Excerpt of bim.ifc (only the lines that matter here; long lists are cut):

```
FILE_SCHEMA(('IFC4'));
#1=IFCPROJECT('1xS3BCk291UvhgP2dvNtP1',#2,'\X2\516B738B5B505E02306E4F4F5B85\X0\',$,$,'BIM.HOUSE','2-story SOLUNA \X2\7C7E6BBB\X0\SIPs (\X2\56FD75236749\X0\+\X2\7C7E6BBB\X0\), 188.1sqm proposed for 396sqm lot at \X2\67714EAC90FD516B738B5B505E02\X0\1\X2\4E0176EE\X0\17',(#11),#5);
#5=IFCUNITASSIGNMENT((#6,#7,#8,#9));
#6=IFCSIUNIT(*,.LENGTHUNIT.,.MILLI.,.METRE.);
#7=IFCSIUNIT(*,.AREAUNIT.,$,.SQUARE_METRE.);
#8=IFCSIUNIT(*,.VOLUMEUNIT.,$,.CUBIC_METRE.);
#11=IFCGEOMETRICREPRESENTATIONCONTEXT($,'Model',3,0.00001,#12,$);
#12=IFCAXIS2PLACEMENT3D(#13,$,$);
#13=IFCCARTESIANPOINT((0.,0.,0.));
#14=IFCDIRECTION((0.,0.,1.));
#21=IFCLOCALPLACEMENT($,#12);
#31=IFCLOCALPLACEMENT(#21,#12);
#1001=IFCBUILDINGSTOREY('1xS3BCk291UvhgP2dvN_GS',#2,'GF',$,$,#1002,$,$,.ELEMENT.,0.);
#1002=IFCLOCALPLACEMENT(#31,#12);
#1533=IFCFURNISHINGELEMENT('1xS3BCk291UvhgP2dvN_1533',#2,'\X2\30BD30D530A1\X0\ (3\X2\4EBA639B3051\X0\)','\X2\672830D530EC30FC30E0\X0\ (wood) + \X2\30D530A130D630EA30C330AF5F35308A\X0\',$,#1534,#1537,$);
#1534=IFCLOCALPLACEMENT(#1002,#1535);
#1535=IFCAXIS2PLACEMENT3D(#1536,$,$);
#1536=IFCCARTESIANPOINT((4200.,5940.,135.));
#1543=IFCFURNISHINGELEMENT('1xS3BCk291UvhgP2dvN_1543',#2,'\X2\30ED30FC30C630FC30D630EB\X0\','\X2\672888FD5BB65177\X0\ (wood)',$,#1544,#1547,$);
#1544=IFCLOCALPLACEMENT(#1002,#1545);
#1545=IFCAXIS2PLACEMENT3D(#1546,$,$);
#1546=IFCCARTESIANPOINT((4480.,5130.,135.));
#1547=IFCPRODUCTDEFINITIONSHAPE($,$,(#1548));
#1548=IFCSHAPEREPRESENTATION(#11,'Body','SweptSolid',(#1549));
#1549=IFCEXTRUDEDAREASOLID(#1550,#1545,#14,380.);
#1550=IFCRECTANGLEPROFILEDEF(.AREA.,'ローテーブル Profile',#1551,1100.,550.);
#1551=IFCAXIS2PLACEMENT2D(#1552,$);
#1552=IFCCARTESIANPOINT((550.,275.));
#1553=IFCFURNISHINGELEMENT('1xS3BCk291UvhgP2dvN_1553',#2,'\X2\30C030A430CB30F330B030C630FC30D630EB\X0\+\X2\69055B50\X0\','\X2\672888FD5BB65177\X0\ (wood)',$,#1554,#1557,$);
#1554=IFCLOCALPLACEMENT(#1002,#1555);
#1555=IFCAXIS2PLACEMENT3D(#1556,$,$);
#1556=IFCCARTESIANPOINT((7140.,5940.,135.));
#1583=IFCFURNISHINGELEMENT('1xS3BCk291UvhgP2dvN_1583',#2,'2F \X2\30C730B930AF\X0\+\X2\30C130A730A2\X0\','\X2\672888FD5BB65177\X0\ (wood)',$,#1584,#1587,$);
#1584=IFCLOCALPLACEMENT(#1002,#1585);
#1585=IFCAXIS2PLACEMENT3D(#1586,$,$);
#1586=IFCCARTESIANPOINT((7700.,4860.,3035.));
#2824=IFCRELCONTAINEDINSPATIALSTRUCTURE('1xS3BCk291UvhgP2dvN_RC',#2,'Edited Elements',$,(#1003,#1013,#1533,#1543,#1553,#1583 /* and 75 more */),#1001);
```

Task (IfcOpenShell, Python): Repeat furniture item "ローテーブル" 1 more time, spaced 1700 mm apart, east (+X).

```python
import numpy as np
import ifcopenshell
import ifcopenshell.api.geometry
import ifcopenshell.api.root
import ifcopenshell.util.element
import ifcopenshell.util.placement
import ifcopenshell.util.unit

model = ifcopenshell.open("bim.ifc")
unit_scale = ifcopenshell.util.unit.calculate_unit_scale(model)


def reuse_history(source, copy):
    """copy_class also copies each property set's owner history, people and application; keep the originals."""
    for rel in copy.IsDefinedBy:
        if rel.is_a("IfcRelDefinesByProperties") and (history := rel.RelatingPropertyDefinition.OwnerHistory):
            rel.RelatingPropertyDefinition.OwnerHistory = source.OwnerHistory
            ifcopenshell.util.element.remove_deep2(model, history)


source = model.by_id(1543)
base = ifcopenshell.util.placement.get_local_placement(source.ObjectPlacement)
step = np.array([1.0, 0.0, 0.0]) * 1.7 / unit_scale

for i in range(1, 2):
    copy = ifcopenshell.api.root.copy_class(model, product=source)
    copy.Representation = ifcopenshell.util.element.copy_deep(
        model, source.Representation, exclude=["IfcGeometricRepresentationContext", "IfcRepresentationMap"]
    )
    reuse_history(source, copy)
    matrix = base.copy()
    matrix[:3, 3] += i * step
    print("added at", matrix[:3, 3].round(3) + 0.0)
    ifcopenshell.api.geometry.edit_object_placement(model, product=copy, matrix=matrix, is_si=False)

model.write("bim_edited.ifc")
```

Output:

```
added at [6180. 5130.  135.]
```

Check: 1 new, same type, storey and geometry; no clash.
